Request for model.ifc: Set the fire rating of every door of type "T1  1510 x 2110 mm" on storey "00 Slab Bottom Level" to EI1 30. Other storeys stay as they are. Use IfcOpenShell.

First a look at what the model holds.

```python
import ifcopenshell
import ifcopenshell.util.element

model = ifcopenshell.open("model.ifc")
print(model.schema)
storey = next(s for s in model.by_type("IfcBuildingStorey") if s.Name == "00 Slab Bottom Level")
doors = [e for e in ifcopenshell.util.element.get_decomposition(storey) if e.is_a("IfcDoor")]
seen = {}
for e in doors:
    element_type = ifcopenshell.util.element.get_type(e)
    key = (element_type.Name if element_type != e and element_type else None, ifcopenshell.util.element.get_pset(e, "Pset_DoorCommon", "FireRating"))
    seen[key] = seen.get(key, 0) + 1
for (name, value), count in sorted(seen.items(), key=str):
    print(count, "x", name, "|", value)
```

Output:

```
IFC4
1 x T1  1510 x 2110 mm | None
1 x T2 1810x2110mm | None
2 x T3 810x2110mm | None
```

```python
import ifcopenshell
import ifcopenshell.api.pset
import ifcopenshell.util.element

model = ifcopenshell.open("model.ifc")

storey = next(s for s in model.by_type("IfcBuildingStorey") if s.Name == "00 Slab Bottom Level")
doors = [e for e in ifcopenshell.util.element.get_decomposition(storey) if e.is_a("IfcDoor")]

count = 0
for e in doors:
    element_type = ifcopenshell.util.element.get_type(e)
    if element_type in (None, e) or element_type.Name != "T1  1510 x 2110 mm":
        continue
    # add_pset returns the element's existing set when there is one.
    pset = ifcopenshell.api.pset.add_pset(model, product=e, name="Pset_DoorCommon")
    ifcopenshell.api.pset.edit_pset(model, pset=pset, properties={"FireRating": "EI1 30"})
    count += 1

print(count, "doors updated")

model.write("model_updated.ifc")
```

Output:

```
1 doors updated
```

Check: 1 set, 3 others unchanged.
